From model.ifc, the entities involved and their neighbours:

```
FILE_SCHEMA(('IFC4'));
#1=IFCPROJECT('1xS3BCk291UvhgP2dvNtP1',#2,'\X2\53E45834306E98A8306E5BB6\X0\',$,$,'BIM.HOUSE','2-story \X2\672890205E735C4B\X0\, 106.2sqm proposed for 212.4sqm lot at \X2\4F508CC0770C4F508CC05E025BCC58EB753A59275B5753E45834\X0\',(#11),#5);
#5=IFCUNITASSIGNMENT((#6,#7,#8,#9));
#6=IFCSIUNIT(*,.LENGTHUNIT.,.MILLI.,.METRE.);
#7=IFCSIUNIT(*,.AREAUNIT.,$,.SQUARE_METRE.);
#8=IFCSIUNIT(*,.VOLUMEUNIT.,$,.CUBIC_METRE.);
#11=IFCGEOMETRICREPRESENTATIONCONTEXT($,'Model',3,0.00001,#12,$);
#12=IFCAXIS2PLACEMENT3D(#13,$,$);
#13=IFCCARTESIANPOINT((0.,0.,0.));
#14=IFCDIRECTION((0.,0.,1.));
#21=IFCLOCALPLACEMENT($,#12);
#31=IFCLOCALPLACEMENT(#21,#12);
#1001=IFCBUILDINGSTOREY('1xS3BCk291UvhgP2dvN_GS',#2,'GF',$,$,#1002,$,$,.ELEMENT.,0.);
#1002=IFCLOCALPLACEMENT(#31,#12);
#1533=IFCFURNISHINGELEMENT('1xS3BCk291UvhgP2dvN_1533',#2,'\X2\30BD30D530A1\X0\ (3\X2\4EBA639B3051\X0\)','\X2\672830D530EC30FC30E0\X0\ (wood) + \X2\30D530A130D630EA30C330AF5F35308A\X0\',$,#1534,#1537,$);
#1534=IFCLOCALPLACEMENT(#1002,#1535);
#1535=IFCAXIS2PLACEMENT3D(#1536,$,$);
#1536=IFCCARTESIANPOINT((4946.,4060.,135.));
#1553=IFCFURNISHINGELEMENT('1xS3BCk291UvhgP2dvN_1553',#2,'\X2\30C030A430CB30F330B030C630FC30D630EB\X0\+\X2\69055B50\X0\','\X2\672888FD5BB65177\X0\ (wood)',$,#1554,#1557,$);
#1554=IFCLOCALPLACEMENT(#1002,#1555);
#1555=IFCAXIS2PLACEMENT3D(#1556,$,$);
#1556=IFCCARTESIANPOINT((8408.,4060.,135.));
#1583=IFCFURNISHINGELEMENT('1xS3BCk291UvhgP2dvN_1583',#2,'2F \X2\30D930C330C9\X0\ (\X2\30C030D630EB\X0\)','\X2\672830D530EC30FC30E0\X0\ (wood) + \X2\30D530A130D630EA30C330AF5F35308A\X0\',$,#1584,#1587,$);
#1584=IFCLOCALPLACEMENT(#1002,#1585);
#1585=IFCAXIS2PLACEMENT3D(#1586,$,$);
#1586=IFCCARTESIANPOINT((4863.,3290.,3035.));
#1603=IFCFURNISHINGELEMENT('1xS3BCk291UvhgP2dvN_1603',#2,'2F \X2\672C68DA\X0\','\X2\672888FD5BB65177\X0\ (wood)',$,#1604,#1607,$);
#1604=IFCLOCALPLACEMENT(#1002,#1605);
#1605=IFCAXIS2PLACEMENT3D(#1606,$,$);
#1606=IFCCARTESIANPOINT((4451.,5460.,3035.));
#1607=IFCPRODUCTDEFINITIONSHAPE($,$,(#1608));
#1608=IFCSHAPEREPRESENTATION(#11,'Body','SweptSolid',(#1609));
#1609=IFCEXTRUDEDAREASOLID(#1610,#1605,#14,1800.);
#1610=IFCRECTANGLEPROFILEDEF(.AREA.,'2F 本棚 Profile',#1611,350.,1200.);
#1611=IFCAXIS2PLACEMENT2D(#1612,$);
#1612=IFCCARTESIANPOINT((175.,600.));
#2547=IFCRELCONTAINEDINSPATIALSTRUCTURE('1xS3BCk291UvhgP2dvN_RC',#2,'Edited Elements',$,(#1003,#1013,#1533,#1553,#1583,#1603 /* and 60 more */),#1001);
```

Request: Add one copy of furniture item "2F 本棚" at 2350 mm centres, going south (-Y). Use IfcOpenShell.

```python
import numpy as np
import ifcopenshell
import ifcopenshell.api.geometry
import ifcopenshell.api.root
import ifcopenshell.util.element
import ifcopenshell.util.placement
import ifcopenshell.util.unit

model = ifcopenshell.open("model.ifc")
unit_scale = ifcopenshell.util.unit.calculate_unit_scale(model)


def reuse_history(source, copy):
    """copy_class also copies each property set's owner history, people and application; keep the originals."""
    for rel in copy.IsDefinedBy:
        if rel.is_a("IfcRelDefinesByProperties") and (history := rel.RelatingPropertyDefinition.OwnerHistory):
            rel.RelatingPropertyDefinition.OwnerHistory = source.OwnerHistory
            ifcopenshell.util.element.remove_deep2(model, history)


source = model.by_guid("1xS3BCk291UvhgP2dvN_1603")
base = ifcopenshell.util.placement.get_local_placement(source.ObjectPlacement)
step = np.array([0.0, -1.0, 0.0]) * 2.35 / unit_scale

for i in range(1, 2):
    copy = ifcopenshell.api.root.copy_class(model, product=source)
    copy.Representation = ifcopenshell.util.element.copy_deep(
        model, source.Representation, exclude=["IfcGeometricRepresentationContext", "IfcRepresentationMap"]
    )
    reuse_history(source, copy)
    matrix = base.copy()
    matrix[:3, 3] += i * step
    print("added at", matrix[:3, 3].round(3) + 0.0)
    ifcopenshell.api.geometry.edit_object_placement(model, product=copy, matrix=matrix, is_si=False)

model.write("model_rev.ifc")
```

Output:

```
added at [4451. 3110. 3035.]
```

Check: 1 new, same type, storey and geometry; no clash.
